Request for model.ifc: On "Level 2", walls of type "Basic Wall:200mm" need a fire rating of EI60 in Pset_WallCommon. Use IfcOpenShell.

First a look at what the model holds.

```python
import ifcopenshell
import ifcopenshell.util.element

model = ifcopenshell.open("model.ifc")
print(model.schema)
storey = next(s for s in model.by_type("IfcBuildingStorey") if s.Name == "Level 2")
walls = [e for e in ifcopenshell.util.element.get_decomposition(storey) if e.is_a("IfcWall")]
seen = {}
for e in walls:
    element_type = ifcopenshell.util.element.get_type(e)
    key = (element_type.Name if element_type != e and element_type else None, ifcopenshell.util.element.get_pset(e, "Pset_WallCommon", "FireRating"))
    seen[key] = seen.get(key, 0) + 1
for (name, value), count in sorted(seen.items(), key=str):
    print(count, "x", name, "|", value)
```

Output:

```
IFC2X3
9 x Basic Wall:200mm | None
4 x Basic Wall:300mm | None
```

```python
import ifcopenshell
import ifcopenshell.api.pset
import ifcopenshell.util.element

model = ifcopenshell.open("model.ifc")

storey = next(s for s in model.by_type("IfcBuildingStorey") if s.Name == "Level 2")
walls = [e for e in ifcopenshell.util.element.get_decomposition(storey) if e.is_a("IfcWall")]

count = 0
for e in walls:
    element_type = ifcopenshell.util.element.get_type(e)
    if element_type in (None, e) or element_type.Name != "Basic Wall:200mm":
        continue
    # add_pset returns the element's existing set when there is one.
    pset = ifcopenshell.api.pset.add_pset(model, product=e, name="Pset_WallCommon")
    ifcopenshell.api.pset.edit_pset(model, pset=pset, properties={"FireRating": "EI60"})
    count += 1

print(count, "walls updated")

model.write("model_updated.ifc")
```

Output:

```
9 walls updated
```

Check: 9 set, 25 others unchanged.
